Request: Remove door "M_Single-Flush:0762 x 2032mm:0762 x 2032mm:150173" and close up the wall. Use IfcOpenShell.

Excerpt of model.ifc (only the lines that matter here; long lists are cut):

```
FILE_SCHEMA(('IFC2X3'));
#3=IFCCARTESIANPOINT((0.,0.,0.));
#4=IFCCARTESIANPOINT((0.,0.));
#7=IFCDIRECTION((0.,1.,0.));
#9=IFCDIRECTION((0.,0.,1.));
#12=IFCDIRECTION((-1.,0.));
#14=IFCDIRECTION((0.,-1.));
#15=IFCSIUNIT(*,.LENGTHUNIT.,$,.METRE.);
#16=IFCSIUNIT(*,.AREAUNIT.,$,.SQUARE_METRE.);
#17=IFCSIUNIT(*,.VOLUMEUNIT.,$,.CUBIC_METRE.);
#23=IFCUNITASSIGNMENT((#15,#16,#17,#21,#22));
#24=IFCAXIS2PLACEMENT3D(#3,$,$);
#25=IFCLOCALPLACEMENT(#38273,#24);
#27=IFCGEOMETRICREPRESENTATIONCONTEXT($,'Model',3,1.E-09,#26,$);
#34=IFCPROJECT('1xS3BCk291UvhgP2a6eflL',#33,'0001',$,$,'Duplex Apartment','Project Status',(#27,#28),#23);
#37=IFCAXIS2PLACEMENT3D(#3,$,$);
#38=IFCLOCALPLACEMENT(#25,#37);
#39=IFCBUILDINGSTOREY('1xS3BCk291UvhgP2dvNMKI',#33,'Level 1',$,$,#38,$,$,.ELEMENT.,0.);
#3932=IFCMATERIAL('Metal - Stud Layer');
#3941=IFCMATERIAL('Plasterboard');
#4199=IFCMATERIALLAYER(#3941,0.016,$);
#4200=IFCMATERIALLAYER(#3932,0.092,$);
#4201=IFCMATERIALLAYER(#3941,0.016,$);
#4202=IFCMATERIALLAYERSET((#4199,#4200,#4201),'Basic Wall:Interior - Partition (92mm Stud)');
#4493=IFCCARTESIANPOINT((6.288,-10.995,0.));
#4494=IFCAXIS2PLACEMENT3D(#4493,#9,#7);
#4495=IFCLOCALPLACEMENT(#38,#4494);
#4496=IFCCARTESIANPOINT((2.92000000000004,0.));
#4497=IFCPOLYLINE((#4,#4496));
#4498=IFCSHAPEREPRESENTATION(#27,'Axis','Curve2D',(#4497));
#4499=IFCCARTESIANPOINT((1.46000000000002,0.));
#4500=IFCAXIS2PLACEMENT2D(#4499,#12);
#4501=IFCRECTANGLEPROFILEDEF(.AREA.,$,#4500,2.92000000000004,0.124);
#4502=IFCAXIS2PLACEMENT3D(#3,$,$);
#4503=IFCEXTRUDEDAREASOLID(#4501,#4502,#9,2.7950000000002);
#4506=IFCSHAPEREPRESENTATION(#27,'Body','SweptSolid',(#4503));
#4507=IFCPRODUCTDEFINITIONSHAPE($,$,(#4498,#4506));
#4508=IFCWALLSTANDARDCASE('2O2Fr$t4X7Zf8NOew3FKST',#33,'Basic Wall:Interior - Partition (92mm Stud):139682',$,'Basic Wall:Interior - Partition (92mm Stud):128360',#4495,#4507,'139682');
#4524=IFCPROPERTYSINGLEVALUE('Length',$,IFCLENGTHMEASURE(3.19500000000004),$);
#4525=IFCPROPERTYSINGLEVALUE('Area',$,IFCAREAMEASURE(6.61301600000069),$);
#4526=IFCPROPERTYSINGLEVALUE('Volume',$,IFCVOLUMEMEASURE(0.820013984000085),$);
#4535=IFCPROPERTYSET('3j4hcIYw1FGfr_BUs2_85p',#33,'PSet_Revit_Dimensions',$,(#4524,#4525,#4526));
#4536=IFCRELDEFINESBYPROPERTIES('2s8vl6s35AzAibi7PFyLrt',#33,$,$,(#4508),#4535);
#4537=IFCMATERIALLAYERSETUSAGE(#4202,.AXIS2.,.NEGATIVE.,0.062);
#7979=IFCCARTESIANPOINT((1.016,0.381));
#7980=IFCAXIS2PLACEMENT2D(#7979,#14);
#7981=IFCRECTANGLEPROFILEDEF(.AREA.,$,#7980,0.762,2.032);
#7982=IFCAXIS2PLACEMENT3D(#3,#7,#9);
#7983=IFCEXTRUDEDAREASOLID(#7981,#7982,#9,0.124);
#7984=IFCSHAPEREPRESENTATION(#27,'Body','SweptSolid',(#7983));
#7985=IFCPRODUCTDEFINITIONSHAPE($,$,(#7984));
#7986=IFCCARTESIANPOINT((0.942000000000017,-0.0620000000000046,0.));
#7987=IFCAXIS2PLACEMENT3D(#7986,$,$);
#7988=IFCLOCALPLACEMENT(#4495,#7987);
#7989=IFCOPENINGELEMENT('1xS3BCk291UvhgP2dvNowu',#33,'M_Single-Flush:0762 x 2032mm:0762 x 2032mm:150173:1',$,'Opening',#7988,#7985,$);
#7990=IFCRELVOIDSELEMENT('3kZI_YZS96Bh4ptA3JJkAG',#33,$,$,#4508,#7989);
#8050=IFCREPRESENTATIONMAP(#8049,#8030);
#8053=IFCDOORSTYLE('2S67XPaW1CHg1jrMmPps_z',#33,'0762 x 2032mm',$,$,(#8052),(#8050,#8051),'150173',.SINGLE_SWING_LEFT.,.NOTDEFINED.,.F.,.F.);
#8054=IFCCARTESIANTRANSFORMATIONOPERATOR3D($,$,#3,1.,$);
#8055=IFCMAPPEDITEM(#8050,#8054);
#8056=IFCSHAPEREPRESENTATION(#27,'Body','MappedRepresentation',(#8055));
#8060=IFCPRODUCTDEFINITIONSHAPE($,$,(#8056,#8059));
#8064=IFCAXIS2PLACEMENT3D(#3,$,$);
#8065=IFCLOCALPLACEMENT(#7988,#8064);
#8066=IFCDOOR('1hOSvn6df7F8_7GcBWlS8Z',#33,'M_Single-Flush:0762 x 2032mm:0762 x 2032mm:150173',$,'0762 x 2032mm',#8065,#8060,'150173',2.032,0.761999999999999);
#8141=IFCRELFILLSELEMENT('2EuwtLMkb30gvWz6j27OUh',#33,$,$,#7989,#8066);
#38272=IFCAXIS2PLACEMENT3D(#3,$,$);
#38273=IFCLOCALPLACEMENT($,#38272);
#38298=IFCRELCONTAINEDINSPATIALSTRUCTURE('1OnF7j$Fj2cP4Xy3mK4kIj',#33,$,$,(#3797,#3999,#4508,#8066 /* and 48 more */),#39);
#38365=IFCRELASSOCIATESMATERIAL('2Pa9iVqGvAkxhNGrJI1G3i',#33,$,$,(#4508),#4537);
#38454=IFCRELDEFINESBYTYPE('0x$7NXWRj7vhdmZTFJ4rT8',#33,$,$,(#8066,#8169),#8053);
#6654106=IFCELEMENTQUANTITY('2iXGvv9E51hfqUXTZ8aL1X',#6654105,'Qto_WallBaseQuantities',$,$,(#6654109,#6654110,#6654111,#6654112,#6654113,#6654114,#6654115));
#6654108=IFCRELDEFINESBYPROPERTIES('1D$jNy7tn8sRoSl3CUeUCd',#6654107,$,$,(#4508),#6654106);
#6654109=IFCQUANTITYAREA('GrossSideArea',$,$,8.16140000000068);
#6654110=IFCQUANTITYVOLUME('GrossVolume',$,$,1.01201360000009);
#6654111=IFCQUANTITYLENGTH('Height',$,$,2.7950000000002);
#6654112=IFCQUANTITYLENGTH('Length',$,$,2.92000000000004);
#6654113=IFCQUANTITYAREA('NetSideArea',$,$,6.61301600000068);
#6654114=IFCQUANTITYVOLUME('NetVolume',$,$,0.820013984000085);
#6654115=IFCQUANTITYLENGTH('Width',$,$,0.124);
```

```python
import ifcopenshell
import ifcopenshell.api.feature
import ifcopenshell.api.pset
import ifcopenshell.api.root
import ifcopenshell.geom
import ifcopenshell.util.element
import ifcopenshell.util.shape
import ifcopenshell.util.unit

model = ifcopenshell.open("model.ifc")
area_scale = ifcopenshell.util.unit.calculate_unit_scale(model, "AREAUNIT")
volume_scale = ifcopenshell.util.unit.calculate_unit_scale(model, "VOLUMEUNIT")
settings = ifcopenshell.geom.settings()


def volume(element):
    """Net volume in cubic metres, openings subtracted."""
    shape = ifcopenshell.geom.create_shape(settings, element)
    return ifcopenshell.util.shape.get_volume(shape.geometry)


door = model.by_guid("1hOSvn6df7F8_7GcBWlS8Z")
opening = door.FillsVoids[0].RelatingOpeningElement
wall = opening.VoidsElements[0].RelatingBuildingElement
before = volume(wall)

ifcopenshell.api.root.remove_product(model, product=door)
ifcopenshell.api.feature.remove_feature(model, feature=opening)

after = volume(wall)
thickness = 0.124  # wall thickness in metres

# Update the wall's stored quantities.
pset = model.by_id(ifcopenshell.util.element.get_pset(wall, "PSet_Revit_Dimensions", should_inherit=False)["id"])
ifcopenshell.api.pset.edit_pset(model, pset=pset, properties={
    "Area": model.create_entity("IfcAreaMeasure", after / thickness / area_scale),
    "Volume": model.create_entity("IfcVolumeMeasure", after / volume_scale),
})
qto = model.by_id(ifcopenshell.util.element.get_pset(wall, "Qto_WallBaseQuantities", should_inherit=False)["id"])
ifcopenshell.api.pset.edit_qto(model, qto=qto, properties={
    "NetSideArea": after / thickness / area_scale,
    "NetVolume": after / volume_scale,
})

print(f"wall volume {before:.3f} -> {after:.3f} m3")

model.write("model_updated.ifc")
```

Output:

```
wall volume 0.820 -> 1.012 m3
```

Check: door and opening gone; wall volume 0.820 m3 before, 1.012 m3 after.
